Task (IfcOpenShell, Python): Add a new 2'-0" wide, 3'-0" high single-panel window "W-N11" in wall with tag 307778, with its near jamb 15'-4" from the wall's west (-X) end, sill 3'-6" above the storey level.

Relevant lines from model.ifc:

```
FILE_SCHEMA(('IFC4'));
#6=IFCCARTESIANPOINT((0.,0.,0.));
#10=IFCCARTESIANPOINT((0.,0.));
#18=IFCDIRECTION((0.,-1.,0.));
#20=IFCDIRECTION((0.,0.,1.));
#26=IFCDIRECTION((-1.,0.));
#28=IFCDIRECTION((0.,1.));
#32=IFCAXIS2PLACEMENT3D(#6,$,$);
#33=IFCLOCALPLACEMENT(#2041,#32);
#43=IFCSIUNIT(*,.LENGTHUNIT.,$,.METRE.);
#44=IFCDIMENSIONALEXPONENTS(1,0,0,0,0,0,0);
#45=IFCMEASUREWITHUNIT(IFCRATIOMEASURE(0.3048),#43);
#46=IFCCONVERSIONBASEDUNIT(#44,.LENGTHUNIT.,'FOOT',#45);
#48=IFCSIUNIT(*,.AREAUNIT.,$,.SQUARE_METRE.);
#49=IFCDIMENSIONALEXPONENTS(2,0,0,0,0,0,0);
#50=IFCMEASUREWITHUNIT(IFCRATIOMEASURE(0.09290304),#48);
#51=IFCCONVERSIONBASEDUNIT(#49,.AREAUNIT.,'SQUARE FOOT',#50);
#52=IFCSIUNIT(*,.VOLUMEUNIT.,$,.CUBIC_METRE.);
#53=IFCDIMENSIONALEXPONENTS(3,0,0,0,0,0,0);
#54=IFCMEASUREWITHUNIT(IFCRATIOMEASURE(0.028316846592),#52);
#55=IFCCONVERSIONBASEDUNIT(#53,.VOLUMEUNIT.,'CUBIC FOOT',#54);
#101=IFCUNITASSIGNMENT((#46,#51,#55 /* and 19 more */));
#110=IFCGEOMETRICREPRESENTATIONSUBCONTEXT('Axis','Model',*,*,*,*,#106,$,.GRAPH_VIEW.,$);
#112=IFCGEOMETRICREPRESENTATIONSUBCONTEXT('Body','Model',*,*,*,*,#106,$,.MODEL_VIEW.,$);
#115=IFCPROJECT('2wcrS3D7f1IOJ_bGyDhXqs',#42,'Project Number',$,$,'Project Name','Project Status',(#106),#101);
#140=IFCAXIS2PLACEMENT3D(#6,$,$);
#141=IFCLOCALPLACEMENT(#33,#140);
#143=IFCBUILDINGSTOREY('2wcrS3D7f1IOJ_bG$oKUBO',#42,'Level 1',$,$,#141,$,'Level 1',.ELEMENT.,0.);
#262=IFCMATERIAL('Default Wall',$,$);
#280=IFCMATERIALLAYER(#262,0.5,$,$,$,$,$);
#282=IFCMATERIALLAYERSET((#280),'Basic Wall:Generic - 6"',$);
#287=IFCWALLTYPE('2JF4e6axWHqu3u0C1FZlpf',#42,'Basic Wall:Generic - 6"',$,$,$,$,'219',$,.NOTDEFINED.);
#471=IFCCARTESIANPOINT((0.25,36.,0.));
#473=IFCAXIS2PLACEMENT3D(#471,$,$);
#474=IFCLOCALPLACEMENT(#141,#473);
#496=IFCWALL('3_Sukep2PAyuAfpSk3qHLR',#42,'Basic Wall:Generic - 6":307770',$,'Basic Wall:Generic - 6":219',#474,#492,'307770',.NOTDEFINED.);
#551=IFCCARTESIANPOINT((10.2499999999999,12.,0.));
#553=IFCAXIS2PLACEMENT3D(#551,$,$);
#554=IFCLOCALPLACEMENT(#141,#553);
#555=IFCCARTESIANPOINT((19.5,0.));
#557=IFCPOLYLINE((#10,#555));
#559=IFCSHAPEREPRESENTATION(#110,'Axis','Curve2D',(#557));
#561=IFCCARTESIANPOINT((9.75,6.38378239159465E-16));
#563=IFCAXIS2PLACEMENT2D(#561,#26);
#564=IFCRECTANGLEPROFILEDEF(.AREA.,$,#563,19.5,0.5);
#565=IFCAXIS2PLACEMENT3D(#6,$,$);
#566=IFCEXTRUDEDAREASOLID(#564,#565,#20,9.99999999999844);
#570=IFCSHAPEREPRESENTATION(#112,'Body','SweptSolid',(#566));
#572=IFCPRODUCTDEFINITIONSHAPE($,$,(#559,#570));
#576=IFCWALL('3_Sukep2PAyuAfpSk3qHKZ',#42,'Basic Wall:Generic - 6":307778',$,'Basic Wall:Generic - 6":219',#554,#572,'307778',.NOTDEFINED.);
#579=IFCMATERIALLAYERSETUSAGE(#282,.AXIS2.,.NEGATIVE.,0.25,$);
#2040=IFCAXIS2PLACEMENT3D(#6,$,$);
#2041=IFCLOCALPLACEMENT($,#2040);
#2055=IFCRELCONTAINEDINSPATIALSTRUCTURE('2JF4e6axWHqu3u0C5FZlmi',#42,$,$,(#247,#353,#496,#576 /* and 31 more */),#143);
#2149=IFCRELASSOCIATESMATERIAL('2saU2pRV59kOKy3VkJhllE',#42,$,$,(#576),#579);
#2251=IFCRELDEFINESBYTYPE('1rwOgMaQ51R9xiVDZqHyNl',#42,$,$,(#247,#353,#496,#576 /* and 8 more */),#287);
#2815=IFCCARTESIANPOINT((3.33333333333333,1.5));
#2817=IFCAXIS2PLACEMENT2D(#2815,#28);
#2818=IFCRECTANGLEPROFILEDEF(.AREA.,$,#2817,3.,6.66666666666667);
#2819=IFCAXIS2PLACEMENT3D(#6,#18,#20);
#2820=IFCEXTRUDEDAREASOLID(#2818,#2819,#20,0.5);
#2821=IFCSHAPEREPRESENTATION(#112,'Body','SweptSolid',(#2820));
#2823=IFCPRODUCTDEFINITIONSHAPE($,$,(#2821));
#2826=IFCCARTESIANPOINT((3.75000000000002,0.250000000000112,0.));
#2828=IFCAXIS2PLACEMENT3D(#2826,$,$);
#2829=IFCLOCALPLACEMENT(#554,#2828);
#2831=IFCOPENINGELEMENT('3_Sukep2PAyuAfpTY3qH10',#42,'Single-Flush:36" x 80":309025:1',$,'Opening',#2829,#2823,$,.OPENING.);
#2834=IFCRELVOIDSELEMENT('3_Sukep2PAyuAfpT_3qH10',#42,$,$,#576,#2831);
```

```python
import numpy as np
import ifcopenshell
import ifcopenshell.api.feature
import ifcopenshell.api.geometry
import ifcopenshell.api.root
import ifcopenshell.api.spatial
import ifcopenshell.geom
import ifcopenshell.util.element
import ifcopenshell.util.placement
import ifcopenshell.util.representation
import ifcopenshell.util.shape
import ifcopenshell.util.unit

model = ifcopenshell.open("model.ifc")
unit_scale = ifcopenshell.util.unit.calculate_unit_scale(model)
settings = ifcopenshell.geom.settings()


def volume(element):
    """Net volume in cubic metres, openings subtracted."""
    shape = ifcopenshell.geom.create_shape(settings, element)
    return ifcopenshell.util.shape.get_volume(shape.geometry)


wall = model.by_guid("3_Sukep2PAyuAfpSk3qHKZ")
storey = ifcopenshell.util.element.get_container(wall, ifc_class="IfcBuildingStorey")
context = ifcopenshell.util.representation.get_context(model, "Model", "Body", "MODEL_VIEW")
before = volume(wall)

width, height, from_end, sill = 0.6096, 0.9144, 4.6736, 1.0668  # metres

# The wall runs along its own X axis, and the end named is its -X end.
wall_shape = ifcopenshell.geom.create_shape(settings, wall)
x, y, z = ifcopenshell.util.shape.get_vertices(wall_shape.geometry).T
start = x.min() + from_end
face, thickness = float(y.min()), float(y.max() - y.min())
wall_matrix = ifcopenshell.util.placement.get_local_placement(wall.ObjectPlacement)
level = ifcopenshell.util.placement.get_local_placement(storey.ObjectPlacement)[2, 3]


def in_wall(x, y):
    """Placement at x, y metres in the wall's axes, at sill height."""
    matrix = wall_matrix.copy()
    matrix[:, 3] = wall_matrix @ np.array([x / unit_scale, y / unit_scale, 0.0, 1.0])
    matrix[2, 3] = level + sill / unit_scale
    return matrix


# Opening: a box that overshoots both wall faces by 50 mm.
opening = ifcopenshell.api.root.create_entity(model, ifc_class="IfcOpeningElement", predefined_type="OPENING")
box = ifcopenshell.api.geometry.add_wall_representation(
    model, context=context, length=width, height=height, thickness=thickness + 0.1
)
ifcopenshell.api.geometry.assign_representation(model, product=opening, representation=box)
ifcopenshell.api.geometry.edit_object_placement(model, product=opening, matrix=in_wall(start, face - 0.05), is_si=False)
ifcopenshell.api.feature.add_feature(model, feature=opening, element=wall)

window = ifcopenshell.api.root.create_entity(model, ifc_class="IfcWindow", name="W-N11", predefined_type="WINDOW")
window.OverallWidth, window.OverallHeight = width / unit_scale, height / unit_scale
window.PartitioningType = "SINGLE_PANEL"
body = ifcopenshell.api.geometry.add_window_representation(
    model,
    context=context,
    overall_width=window.OverallWidth,
    overall_height=window.OverallHeight,
    partition_type="SINGLE_PANEL",
)
ifcopenshell.api.geometry.assign_representation(model, product=window, representation=body)
ifcopenshell.api.spatial.assign_container(model, products=[window], relating_structure=storey)
ifcopenshell.api.feature.add_filling(model, opening=opening, element=window)

# Centre the window in the wall's thickness.
ifcopenshell.api.geometry.edit_object_placement(model, product=window, matrix=in_wall(start, face), is_si=False)
window_shape = ifcopenshell.geom.create_shape(settings, window)
depth = ifcopenshell.util.shape.get_vertices(window_shape.geometry)[:, 1]
offset = face + thickness / 2 - (depth.min() + depth.max()) / 2
ifcopenshell.api.geometry.edit_object_placement(model, product=window, matrix=in_wall(start, offset), is_si=False)

after = volume(wall)

print(f"wall volume {before:.3f} -> {after:.3f} m3")

model.write("model_updated.ifc")
```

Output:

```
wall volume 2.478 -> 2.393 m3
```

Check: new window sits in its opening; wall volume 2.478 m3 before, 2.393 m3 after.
